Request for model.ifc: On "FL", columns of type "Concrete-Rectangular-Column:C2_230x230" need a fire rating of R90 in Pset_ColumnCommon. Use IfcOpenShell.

First a look at what the model holds.

```python
import ifcopenshell
import ifcopenshell.util.element

model = ifcopenshell.open("model.ifc")
print(model.schema)
storey = next(s for s in model.by_type("IfcBuildingStorey") if s.Name == "FL")
columns = [e for e in ifcopenshell.util.element.get_decomposition(storey) if e.is_a("IfcColumn")]
seen = {}
for e in columns:
    element_type = ifcopenshell.util.element.get_type(e)
    key = (element_type.Name if element_type != e and element_type else None, ifcopenshell.util.element.get_pset(e, "Pset_ColumnCommon", "FireRating"))
    seen[key] = seen.get(key, 0) + 1
for (name, value), count in sorted(seen.items(), key=str):
    print(count, "x", name, "|", value)
```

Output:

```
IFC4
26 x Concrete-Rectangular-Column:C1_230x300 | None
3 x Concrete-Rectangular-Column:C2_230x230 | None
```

```python
import ifcopenshell
import ifcopenshell.api.pset
import ifcopenshell.util.element

model = ifcopenshell.open("model.ifc")

storey = next(s for s in model.by_type("IfcBuildingStorey") if s.Name == "FL")
columns = [e for e in ifcopenshell.util.element.get_decomposition(storey) if e.is_a("IfcColumn")]

count = 0
for e in columns:
    element_type = ifcopenshell.util.element.get_type(e)
    if element_type in (None, e) or element_type.Name != "Concrete-Rectangular-Column:C2_230x230":
        continue
    # add_pset returns the element's existing set when there is one.
    pset = ifcopenshell.api.pset.add_pset(model, product=e, name="Pset_ColumnCommon")
    ifcopenshell.api.pset.edit_pset(model, pset=pset, properties={"FireRating": "R90"})
    count += 1

print(count, "columns updated")

model.write("model_updated.ifc")
```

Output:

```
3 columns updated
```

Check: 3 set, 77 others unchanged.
